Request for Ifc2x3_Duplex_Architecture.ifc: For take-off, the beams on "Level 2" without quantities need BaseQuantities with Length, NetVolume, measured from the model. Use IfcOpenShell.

First a look at what the model holds.

```python
import ifcopenshell
import ifcopenshell.util.element
import ifcopenshell.util.unit

model = ifcopenshell.open("Ifc2x3_Duplex_Architecture.ifc")
print(model.schema)
for unit_type in ("LENGTHUNIT", "AREAUNIT", "VOLUMEUNIT"):
    print(unit_type, ifcopenshell.util.unit.calculate_unit_scale(model, unit_type))
storey = next(s for s in model.by_type("IfcBuildingStorey") if s.Name == "Level 2")
beams = [e for e in ifcopenshell.util.element.get_decomposition(storey) if e.is_a("IfcBeam")]
for e in sorted(beams, key=lambda e: e.id()):
    print(e.id(), e.is_a(), e.Name, list(ifcopenshell.util.element.get_psets(e, qtos_only=True)), sep=" | ")
```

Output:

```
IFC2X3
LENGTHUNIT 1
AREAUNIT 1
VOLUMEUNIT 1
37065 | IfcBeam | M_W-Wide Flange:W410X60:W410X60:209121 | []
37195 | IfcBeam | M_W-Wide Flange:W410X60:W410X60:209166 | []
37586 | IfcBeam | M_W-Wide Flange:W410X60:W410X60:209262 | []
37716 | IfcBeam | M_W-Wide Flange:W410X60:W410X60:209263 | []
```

```python
import ifcopenshell
import ifcopenshell.api.pset
import ifcopenshell.geom
import ifcopenshell.util.element
import ifcopenshell.util.shape
import ifcopenshell.util.unit

model = ifcopenshell.open("Ifc2x3_Duplex_Architecture.ifc")
unit_scale = ifcopenshell.util.unit.calculate_unit_scale(model)
volume_scale = ifcopenshell.util.unit.calculate_unit_scale(model, "VOLUMEUNIT")
settings = ifcopenshell.geom.settings()

storey = next(s for s in model.by_type("IfcBuildingStorey") if s.Name == "Level 2")
beams = [e for e in ifcopenshell.util.element.get_decomposition(storey) if e.is_a("IfcBeam")]

for e in sorted(beams, key=lambda e: e.id()):
    if ifcopenshell.util.element.get_psets(e, qtos_only=True, should_inherit=False):
        continue
    # Geometry comes back in metres, in the element's own axes.
    shape = ifcopenshell.geom.create_shape(settings, e)
    values = {
        "Length": ifcopenshell.util.shape.get_max_xyz(shape.geometry) / unit_scale,
        "NetVolume": ifcopenshell.util.shape.get_volume(shape.geometry) / volume_scale,
    }
    qto = ifcopenshell.api.pset.add_qto(model, product=e, name="BaseQuantities")
    ifcopenshell.api.pset.edit_qto(model, qto=qto, properties=values)
    print(e.id(), {k: round(v, 3) for k, v in values.items()})

model.write("Ifc2x3_Duplex_Architecture_rev.ifc")
```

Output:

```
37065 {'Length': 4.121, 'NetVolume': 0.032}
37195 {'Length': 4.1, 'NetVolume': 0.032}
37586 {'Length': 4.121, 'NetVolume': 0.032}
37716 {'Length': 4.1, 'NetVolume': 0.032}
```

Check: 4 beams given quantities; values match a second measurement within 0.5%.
